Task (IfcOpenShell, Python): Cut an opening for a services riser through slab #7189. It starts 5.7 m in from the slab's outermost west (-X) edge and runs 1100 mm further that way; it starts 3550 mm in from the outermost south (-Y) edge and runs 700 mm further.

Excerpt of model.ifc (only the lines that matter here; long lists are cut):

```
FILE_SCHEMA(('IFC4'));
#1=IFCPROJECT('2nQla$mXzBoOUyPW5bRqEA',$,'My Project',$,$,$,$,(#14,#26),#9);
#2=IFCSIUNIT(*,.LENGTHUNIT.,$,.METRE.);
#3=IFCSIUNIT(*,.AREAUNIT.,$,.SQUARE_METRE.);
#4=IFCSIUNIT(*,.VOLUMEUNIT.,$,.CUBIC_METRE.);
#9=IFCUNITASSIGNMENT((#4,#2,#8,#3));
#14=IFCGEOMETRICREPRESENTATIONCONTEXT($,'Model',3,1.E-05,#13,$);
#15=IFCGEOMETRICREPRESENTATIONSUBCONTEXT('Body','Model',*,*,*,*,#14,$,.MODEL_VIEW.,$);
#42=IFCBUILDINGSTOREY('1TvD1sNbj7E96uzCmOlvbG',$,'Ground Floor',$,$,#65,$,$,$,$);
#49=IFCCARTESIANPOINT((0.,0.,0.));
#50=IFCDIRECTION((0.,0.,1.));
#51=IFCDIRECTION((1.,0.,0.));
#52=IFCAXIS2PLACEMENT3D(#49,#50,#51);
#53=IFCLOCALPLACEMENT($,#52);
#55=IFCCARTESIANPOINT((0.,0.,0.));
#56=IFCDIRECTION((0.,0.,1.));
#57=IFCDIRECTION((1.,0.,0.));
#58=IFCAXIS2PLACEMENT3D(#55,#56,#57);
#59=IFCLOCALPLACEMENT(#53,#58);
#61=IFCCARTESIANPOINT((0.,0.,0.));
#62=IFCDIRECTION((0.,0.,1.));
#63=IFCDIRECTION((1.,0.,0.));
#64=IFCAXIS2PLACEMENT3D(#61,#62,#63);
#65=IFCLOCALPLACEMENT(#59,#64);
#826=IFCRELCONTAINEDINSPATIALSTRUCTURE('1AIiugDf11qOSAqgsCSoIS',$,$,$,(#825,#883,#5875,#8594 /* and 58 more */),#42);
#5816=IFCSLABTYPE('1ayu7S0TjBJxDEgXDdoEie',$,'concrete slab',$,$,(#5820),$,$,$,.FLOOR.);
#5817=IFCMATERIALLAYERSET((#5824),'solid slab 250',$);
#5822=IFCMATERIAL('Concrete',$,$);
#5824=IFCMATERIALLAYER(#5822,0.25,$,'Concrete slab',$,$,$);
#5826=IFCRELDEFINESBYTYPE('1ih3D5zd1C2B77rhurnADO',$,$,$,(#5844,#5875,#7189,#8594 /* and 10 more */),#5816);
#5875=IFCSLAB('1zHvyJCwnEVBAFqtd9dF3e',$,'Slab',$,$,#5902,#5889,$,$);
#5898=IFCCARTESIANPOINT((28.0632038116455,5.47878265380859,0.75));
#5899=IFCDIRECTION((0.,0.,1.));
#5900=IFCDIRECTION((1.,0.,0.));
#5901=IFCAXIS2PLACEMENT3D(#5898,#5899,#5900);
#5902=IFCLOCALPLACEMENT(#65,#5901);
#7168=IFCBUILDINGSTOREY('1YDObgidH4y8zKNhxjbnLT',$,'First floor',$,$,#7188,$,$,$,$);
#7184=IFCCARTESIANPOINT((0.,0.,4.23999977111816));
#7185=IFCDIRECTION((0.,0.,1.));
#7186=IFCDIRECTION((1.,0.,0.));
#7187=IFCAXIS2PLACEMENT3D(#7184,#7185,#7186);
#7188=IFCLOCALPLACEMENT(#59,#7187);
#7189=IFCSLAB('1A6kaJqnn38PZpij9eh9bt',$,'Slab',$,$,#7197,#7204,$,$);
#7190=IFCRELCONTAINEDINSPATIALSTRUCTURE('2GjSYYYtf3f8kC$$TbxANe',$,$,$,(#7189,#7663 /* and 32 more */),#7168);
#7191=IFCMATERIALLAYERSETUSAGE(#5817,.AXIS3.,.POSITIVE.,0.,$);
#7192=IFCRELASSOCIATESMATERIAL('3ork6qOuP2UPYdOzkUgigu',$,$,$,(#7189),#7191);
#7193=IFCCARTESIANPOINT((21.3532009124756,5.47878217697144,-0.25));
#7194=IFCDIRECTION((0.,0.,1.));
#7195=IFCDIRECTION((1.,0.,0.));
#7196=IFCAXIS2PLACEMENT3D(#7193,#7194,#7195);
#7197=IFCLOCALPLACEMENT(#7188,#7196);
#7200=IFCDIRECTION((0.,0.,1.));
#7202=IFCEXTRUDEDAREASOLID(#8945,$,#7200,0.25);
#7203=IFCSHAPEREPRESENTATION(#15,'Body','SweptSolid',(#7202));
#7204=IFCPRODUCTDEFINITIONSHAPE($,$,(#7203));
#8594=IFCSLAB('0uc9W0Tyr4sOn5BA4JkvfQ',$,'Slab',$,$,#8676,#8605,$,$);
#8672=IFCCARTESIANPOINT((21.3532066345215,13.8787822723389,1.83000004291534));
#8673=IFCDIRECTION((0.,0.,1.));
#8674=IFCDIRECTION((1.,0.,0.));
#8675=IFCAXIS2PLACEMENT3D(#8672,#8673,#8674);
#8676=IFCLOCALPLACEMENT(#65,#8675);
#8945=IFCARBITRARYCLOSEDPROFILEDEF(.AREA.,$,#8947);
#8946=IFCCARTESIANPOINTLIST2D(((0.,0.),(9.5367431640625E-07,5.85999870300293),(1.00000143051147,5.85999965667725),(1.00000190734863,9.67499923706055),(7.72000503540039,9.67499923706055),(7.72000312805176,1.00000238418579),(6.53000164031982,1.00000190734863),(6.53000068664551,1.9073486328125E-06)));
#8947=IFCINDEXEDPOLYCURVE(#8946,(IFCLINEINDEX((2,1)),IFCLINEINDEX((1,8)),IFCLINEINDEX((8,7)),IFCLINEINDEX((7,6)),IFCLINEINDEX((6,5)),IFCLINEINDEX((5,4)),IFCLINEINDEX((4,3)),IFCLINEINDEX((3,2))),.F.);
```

```python
import numpy as np
import ifcopenshell
import ifcopenshell.api.feature
import ifcopenshell.api.geometry
import ifcopenshell.api.root
import ifcopenshell.geom
import ifcopenshell.util.placement
import ifcopenshell.util.representation
import ifcopenshell.util.shape
import ifcopenshell.util.unit

model = ifcopenshell.open("model.ifc")
unit_scale = ifcopenshell.util.unit.calculate_unit_scale(model)
settings = ifcopenshell.geom.settings()


def volume(element):
    """Net volume in cubic metres, openings subtracted."""
    shape = ifcopenshell.geom.create_shape(settings, element)
    return ifcopenshell.util.shape.get_volume(shape.geometry)


slab = model.by_guid("1A6kaJqnn38PZpij9eh9bt")
before = volume(slab)

# Extent in the slab's own axes, in metres. The edges named are its -X and -Y sides.
slab_shape = ifcopenshell.geom.create_shape(settings, slab)
vertices = ifcopenshell.util.shape.get_vertices(slab_shape.geometry)
x_min, y_min, bottom = vertices.min(axis=0)
top = vertices[:, 2].max()

opening = ifcopenshell.api.root.create_entity(model, ifc_class="IfcOpeningElement", name="Services riser opening", predefined_type="OPENING")
context = ifcopenshell.util.representation.get_context(model, "Model", "Body", "MODEL_VIEW")
width, depth = 1.1, 0.7
outline = [(0.0, 0.0), (width, 0.0), (width, depth), (0.0, depth), (0.0, 0.0)]
# Overshoot both faces by 50 mm so the cut is clean.
shape = ifcopenshell.api.geometry.add_slab_representation(
    model, context=context, depth=top - bottom + 0.1, polyline=outline
)
ifcopenshell.api.geometry.assign_representation(model, product=opening, representation=shape)

matrix = ifcopenshell.util.placement.get_local_placement(slab.ObjectPlacement)
matrix[:, 3] = matrix @ np.append(np.array([x_min + 5.7, y_min + 3.55, bottom - 0.05]) / unit_scale, 1.0)
ifcopenshell.api.geometry.edit_object_placement(model, product=opening, matrix=matrix, is_si=False)
ifcopenshell.api.feature.add_feature(model, feature=opening, element=slab)

after = volume(slab)

print(f"slab volume {before:.3f} -> {after:.3f} m3")

model.write("model_v2.ifc")
```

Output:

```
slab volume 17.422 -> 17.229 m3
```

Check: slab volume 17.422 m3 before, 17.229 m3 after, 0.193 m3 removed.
